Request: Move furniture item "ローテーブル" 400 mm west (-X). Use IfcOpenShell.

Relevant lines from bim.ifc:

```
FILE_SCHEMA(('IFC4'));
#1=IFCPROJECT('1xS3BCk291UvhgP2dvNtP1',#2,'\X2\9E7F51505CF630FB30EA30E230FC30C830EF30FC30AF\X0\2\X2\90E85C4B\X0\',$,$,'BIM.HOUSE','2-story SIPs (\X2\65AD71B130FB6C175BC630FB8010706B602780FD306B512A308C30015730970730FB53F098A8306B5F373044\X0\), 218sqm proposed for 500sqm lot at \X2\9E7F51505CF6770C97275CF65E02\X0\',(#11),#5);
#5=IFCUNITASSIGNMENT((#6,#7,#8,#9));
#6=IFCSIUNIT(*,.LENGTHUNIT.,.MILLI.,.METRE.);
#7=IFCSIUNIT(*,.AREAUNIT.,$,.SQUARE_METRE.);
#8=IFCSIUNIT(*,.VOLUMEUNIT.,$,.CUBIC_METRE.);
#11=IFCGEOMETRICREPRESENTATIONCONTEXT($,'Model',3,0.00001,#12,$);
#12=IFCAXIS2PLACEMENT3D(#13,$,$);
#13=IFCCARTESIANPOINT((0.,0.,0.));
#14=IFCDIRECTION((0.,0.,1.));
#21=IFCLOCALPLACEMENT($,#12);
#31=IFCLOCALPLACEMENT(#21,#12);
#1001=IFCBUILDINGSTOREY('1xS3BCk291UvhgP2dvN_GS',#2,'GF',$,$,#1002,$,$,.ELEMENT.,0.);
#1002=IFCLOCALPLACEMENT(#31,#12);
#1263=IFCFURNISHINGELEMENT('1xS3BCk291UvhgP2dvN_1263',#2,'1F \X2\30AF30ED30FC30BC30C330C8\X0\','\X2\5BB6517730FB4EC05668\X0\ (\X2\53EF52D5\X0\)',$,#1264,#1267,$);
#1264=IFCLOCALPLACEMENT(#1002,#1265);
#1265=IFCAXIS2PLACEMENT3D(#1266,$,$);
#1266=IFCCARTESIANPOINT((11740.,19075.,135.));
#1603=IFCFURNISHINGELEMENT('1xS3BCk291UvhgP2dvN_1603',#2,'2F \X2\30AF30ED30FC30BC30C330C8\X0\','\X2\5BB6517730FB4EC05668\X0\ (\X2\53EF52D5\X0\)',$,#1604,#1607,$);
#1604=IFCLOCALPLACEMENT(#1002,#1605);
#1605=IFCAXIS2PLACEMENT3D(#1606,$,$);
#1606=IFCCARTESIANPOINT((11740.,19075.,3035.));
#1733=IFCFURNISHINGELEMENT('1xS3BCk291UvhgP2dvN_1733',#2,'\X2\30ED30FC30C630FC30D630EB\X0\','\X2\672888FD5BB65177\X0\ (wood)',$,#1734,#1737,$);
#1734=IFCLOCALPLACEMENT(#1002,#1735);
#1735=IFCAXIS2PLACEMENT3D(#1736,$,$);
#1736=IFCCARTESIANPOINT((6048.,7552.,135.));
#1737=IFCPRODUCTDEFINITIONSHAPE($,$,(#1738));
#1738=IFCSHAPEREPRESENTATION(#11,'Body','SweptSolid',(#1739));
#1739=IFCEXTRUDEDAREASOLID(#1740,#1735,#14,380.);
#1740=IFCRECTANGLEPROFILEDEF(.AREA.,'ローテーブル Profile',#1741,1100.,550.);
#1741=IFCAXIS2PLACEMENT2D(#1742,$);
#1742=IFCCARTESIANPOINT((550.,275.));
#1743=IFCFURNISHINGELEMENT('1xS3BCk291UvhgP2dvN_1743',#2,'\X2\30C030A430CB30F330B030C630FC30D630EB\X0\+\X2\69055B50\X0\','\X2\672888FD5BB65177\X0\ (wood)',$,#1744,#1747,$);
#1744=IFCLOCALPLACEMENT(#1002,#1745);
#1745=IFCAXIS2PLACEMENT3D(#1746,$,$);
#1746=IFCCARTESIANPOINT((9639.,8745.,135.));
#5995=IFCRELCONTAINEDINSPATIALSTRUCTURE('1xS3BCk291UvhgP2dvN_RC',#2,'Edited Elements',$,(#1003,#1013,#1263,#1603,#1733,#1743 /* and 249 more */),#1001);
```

```python
import ifcopenshell
import ifcopenshell.api.geometry
import ifcopenshell.util.placement
import ifcopenshell.util.unit

model = ifcopenshell.open("bim.ifc")
unit_scale = ifcopenshell.util.unit.calculate_unit_scale(model)

item = model.by_guid("1xS3BCk291UvhgP2dvN_1733")
matrix = ifcopenshell.util.placement.get_local_placement(item.ObjectPlacement)
matrix[0, 3] -= 0.4 / unit_scale
ifcopenshell.api.geometry.edit_object_placement(model, product=item, matrix=matrix, is_si=False)

print(ifcopenshell.util.placement.get_local_placement(item.ObjectPlacement).round(3) + 0.0)

model.write("bim-out.ifc")
```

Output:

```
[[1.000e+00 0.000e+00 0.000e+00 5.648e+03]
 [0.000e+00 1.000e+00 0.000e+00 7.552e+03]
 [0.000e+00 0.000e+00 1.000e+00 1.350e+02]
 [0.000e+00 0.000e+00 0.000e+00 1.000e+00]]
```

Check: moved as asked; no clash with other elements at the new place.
